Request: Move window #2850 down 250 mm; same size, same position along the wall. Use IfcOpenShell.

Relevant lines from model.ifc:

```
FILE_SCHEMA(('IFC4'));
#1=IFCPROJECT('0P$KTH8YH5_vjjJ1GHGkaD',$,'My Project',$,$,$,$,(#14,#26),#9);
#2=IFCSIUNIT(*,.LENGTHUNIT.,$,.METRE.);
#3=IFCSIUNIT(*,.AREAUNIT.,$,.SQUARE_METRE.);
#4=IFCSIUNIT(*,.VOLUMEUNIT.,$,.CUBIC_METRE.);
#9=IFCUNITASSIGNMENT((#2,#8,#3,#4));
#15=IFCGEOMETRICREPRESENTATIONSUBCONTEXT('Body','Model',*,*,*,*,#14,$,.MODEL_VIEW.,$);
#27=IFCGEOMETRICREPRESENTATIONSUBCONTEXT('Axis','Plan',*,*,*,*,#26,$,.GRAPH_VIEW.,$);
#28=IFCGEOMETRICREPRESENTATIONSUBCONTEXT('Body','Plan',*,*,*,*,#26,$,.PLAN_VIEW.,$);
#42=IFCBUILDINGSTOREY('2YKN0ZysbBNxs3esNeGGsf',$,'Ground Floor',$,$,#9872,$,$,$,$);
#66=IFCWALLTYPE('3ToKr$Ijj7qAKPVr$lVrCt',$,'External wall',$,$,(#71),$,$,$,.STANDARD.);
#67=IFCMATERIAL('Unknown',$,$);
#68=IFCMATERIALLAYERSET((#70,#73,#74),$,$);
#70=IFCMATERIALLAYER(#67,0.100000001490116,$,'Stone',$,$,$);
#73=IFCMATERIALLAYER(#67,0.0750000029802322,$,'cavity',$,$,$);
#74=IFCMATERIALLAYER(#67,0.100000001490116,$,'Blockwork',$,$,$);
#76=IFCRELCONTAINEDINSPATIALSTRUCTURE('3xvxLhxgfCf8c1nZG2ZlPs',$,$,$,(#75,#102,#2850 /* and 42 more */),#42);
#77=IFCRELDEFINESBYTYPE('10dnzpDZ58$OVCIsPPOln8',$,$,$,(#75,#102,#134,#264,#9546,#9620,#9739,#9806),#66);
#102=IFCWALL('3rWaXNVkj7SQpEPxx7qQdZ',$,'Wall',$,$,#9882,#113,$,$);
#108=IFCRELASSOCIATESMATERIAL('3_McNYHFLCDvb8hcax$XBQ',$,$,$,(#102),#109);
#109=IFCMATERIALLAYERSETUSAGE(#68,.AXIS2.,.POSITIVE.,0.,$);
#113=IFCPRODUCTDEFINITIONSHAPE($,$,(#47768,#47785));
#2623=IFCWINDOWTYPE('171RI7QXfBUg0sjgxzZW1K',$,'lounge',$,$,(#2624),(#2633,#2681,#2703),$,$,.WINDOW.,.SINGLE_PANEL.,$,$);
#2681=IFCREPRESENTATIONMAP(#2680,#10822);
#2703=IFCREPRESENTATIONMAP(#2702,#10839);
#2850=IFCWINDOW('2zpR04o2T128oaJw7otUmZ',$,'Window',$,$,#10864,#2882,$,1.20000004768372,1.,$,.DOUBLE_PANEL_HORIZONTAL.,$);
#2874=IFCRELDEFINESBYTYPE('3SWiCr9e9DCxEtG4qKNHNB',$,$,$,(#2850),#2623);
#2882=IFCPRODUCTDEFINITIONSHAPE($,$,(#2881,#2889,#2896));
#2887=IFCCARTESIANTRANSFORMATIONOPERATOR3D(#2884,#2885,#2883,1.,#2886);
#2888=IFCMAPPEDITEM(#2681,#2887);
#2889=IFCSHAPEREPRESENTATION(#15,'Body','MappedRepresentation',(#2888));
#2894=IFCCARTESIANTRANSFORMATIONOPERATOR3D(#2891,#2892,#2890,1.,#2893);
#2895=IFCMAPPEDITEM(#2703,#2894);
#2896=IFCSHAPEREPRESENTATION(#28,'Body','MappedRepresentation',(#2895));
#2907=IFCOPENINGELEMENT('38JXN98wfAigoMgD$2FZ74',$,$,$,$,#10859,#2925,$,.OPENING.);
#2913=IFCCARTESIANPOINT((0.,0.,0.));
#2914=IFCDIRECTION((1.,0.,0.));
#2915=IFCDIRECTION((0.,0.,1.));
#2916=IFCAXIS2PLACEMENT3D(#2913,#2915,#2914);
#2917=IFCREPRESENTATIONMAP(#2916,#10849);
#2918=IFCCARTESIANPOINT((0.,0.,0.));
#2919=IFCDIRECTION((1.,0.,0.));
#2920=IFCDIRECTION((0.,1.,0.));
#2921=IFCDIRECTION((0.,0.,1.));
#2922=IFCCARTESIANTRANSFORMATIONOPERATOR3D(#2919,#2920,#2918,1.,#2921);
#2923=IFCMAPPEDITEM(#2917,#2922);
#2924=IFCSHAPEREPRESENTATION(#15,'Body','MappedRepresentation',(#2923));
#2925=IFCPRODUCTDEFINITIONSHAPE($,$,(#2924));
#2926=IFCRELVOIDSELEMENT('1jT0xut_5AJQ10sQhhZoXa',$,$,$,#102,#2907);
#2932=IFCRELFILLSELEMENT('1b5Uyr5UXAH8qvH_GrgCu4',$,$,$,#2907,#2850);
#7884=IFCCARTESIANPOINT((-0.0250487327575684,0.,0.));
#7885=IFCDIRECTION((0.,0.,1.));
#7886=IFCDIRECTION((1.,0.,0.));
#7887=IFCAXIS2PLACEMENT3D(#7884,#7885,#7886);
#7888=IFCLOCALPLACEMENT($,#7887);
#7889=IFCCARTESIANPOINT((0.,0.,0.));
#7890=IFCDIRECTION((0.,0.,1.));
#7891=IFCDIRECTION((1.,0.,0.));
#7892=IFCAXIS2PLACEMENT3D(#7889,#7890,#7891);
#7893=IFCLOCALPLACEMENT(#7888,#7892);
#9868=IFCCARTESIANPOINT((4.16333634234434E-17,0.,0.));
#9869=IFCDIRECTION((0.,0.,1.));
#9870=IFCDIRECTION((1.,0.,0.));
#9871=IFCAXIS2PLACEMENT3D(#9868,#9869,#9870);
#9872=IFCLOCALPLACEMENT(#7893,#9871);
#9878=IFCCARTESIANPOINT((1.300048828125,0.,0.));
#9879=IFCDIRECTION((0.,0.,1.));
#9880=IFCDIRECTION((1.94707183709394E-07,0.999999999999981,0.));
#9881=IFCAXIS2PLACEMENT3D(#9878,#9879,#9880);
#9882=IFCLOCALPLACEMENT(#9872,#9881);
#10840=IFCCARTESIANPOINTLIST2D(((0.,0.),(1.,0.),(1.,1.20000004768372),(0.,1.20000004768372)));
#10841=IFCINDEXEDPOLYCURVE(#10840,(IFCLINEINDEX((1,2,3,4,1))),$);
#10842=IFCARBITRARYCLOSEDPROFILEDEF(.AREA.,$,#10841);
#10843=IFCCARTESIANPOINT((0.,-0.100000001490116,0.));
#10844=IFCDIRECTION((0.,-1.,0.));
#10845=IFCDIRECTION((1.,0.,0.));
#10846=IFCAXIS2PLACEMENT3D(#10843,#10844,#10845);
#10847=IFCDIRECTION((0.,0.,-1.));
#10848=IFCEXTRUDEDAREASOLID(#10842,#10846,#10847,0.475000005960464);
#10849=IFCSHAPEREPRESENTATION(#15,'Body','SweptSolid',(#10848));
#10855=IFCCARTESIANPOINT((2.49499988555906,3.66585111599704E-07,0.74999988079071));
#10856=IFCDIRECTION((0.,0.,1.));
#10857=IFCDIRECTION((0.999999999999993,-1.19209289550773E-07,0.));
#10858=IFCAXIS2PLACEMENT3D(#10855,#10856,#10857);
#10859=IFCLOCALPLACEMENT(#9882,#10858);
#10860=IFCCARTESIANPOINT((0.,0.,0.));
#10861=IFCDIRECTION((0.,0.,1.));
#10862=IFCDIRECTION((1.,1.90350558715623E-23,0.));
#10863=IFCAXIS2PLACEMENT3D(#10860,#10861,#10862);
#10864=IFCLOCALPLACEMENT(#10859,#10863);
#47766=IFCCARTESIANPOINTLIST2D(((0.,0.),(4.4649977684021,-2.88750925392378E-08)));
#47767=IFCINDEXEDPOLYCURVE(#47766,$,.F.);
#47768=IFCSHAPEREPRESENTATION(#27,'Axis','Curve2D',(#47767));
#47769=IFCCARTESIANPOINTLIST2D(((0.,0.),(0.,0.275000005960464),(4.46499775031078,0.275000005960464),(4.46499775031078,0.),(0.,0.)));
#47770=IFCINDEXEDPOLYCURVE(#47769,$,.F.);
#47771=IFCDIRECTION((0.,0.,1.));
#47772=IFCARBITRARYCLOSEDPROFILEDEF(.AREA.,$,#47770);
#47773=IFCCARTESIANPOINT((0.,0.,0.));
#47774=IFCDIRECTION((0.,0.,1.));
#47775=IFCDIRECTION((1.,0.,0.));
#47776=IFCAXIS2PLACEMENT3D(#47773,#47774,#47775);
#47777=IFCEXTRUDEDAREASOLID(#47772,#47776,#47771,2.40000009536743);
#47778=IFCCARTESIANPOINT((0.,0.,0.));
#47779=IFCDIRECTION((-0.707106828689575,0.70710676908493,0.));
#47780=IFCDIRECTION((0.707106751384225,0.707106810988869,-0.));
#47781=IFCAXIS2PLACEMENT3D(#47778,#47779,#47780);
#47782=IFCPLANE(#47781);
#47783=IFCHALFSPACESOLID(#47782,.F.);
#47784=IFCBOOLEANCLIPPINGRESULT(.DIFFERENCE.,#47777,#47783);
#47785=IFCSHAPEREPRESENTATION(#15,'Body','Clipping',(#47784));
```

```python
import numpy as np
import ifcopenshell
import ifcopenshell.api.geometry
import ifcopenshell.util.placement
import ifcopenshell.util.unit

model = ifcopenshell.open("model.ifc")
unit_scale = ifcopenshell.util.unit.calculate_unit_scale(model)

window = model.by_guid("2zpR04o2T128oaJw7otUmZ")
opening = window.FillsVoids[0].RelatingOpeningElement
dz = -0.25 / unit_scale

shift = np.array([0.0, 0.0, dz])
# The window is placed relative to its opening, so it follows when the opening moves.
matrix = ifcopenshell.util.placement.get_local_placement(opening.ObjectPlacement)
matrix[:3, 3] += shift
ifcopenshell.api.geometry.edit_object_placement(
    model, product=opening, matrix=matrix, is_si=False, should_transform_children=True
)

print(f"moved by {dz * unit_scale:+.3f} m")

model.write("model-out.ifc")
```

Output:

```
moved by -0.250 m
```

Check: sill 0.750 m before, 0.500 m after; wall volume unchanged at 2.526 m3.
